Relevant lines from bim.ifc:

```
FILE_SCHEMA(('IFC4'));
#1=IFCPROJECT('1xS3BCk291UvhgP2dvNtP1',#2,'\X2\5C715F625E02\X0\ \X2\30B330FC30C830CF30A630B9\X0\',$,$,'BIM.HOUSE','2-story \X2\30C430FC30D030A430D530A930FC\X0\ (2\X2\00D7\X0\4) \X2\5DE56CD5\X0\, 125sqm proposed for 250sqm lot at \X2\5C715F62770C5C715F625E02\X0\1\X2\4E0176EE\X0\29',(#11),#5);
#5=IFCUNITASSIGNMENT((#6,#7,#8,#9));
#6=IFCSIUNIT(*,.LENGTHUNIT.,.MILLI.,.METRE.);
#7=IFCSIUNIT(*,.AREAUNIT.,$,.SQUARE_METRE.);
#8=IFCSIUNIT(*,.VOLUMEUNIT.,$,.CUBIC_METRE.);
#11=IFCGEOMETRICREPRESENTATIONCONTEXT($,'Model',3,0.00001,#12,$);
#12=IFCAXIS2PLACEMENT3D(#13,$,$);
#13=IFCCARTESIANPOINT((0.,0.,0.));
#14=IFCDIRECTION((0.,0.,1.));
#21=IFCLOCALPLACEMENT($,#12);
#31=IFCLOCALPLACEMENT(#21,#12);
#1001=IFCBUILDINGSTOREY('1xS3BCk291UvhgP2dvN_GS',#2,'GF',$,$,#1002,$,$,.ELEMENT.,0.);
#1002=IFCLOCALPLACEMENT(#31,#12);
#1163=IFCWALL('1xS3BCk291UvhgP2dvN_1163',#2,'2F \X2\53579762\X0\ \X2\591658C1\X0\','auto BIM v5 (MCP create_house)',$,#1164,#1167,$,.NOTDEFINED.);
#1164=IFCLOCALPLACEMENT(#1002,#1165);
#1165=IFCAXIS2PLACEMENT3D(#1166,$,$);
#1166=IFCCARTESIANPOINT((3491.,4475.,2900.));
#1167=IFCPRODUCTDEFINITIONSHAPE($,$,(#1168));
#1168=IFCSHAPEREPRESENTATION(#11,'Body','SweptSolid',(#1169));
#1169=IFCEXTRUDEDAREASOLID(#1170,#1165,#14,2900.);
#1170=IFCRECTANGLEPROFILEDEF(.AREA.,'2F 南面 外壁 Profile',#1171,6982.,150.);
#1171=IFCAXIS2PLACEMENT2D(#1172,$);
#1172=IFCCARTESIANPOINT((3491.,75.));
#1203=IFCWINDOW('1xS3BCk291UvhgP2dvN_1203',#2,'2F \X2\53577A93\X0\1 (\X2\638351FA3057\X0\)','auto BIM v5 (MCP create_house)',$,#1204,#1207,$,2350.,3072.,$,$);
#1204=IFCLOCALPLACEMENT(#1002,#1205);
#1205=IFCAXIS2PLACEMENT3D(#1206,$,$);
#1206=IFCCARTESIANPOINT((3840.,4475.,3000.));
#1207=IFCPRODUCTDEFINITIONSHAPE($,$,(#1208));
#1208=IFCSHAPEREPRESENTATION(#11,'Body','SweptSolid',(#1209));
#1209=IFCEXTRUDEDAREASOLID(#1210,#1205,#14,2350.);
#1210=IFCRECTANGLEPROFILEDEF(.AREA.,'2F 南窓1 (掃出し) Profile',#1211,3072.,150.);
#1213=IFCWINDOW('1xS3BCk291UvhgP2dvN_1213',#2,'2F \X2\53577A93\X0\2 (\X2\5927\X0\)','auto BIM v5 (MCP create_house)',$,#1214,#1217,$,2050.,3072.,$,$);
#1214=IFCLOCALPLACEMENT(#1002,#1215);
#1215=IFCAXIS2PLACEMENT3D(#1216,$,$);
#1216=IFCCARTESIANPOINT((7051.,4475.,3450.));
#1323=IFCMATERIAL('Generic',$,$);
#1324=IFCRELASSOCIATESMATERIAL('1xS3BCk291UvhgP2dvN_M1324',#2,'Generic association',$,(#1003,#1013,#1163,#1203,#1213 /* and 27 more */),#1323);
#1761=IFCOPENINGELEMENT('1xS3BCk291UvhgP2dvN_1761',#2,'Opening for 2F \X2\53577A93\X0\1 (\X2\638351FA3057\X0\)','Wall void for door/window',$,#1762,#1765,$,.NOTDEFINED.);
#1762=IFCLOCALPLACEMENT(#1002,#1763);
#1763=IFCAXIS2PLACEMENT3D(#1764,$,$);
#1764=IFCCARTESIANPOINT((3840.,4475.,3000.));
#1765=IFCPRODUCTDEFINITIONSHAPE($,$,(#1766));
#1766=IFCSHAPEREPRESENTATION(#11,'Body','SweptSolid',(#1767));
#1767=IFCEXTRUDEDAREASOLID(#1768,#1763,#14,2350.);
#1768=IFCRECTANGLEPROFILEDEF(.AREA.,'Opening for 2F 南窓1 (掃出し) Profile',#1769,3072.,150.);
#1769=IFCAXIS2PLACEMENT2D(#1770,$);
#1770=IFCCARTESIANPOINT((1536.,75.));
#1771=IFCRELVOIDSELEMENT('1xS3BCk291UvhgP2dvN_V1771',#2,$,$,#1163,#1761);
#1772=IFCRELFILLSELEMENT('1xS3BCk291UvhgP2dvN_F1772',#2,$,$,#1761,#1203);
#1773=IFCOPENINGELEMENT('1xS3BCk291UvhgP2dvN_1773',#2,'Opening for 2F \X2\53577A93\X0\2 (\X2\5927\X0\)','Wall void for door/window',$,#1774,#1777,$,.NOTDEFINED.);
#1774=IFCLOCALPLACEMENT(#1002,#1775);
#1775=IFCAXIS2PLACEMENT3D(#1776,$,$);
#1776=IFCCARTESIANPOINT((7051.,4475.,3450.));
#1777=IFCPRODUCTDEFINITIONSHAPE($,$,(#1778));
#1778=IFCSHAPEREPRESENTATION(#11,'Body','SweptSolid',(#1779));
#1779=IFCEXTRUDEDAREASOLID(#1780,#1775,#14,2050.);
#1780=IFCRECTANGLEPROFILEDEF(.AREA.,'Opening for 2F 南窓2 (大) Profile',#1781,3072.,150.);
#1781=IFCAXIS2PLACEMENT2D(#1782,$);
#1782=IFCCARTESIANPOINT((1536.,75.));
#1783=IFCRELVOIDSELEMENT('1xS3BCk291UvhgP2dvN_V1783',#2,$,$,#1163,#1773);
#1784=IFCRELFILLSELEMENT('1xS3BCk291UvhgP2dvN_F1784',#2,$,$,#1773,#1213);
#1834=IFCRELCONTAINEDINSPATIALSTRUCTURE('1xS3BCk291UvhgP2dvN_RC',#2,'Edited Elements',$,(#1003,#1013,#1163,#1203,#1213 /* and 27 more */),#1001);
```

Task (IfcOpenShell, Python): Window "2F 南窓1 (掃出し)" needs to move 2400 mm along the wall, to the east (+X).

```python
import ifcopenshell
import ifcopenshell.api.geometry
import ifcopenshell.util.placement

model = ifcopenshell.open("bim.ifc")

window = model.by_guid("1xS3BCk291UvhgP2dvN_1203")
opening = window.FillsVoids[0].RelatingOpeningElement
wall = opening.VoidsElements[0].RelatingBuildingElement

wall_matrix = ifcopenshell.util.placement.get_local_placement(wall.ObjectPlacement)
shift = wall_matrix[:3, 0] * 2400.0
before = ifcopenshell.util.placement.get_local_placement(window.ObjectPlacement)[:3, 3].copy()

# The window is not placed relative to its opening, so move both.
for product in (opening, window):
    matrix = ifcopenshell.util.placement.get_local_placement(product.ObjectPlacement)
    matrix[:3, 3] += shift
    ifcopenshell.api.geometry.edit_object_placement(model, product=product, matrix=matrix, is_si=False)

after = ifcopenshell.util.placement.get_local_placement(window.ObjectPlacement)[:3, 3]
print("window moved by", (after - before).round(3) + 0.0)

model.write("bim_updated.ifc")
```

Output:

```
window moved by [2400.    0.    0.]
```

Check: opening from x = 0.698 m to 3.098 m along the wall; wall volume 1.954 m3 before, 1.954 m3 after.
